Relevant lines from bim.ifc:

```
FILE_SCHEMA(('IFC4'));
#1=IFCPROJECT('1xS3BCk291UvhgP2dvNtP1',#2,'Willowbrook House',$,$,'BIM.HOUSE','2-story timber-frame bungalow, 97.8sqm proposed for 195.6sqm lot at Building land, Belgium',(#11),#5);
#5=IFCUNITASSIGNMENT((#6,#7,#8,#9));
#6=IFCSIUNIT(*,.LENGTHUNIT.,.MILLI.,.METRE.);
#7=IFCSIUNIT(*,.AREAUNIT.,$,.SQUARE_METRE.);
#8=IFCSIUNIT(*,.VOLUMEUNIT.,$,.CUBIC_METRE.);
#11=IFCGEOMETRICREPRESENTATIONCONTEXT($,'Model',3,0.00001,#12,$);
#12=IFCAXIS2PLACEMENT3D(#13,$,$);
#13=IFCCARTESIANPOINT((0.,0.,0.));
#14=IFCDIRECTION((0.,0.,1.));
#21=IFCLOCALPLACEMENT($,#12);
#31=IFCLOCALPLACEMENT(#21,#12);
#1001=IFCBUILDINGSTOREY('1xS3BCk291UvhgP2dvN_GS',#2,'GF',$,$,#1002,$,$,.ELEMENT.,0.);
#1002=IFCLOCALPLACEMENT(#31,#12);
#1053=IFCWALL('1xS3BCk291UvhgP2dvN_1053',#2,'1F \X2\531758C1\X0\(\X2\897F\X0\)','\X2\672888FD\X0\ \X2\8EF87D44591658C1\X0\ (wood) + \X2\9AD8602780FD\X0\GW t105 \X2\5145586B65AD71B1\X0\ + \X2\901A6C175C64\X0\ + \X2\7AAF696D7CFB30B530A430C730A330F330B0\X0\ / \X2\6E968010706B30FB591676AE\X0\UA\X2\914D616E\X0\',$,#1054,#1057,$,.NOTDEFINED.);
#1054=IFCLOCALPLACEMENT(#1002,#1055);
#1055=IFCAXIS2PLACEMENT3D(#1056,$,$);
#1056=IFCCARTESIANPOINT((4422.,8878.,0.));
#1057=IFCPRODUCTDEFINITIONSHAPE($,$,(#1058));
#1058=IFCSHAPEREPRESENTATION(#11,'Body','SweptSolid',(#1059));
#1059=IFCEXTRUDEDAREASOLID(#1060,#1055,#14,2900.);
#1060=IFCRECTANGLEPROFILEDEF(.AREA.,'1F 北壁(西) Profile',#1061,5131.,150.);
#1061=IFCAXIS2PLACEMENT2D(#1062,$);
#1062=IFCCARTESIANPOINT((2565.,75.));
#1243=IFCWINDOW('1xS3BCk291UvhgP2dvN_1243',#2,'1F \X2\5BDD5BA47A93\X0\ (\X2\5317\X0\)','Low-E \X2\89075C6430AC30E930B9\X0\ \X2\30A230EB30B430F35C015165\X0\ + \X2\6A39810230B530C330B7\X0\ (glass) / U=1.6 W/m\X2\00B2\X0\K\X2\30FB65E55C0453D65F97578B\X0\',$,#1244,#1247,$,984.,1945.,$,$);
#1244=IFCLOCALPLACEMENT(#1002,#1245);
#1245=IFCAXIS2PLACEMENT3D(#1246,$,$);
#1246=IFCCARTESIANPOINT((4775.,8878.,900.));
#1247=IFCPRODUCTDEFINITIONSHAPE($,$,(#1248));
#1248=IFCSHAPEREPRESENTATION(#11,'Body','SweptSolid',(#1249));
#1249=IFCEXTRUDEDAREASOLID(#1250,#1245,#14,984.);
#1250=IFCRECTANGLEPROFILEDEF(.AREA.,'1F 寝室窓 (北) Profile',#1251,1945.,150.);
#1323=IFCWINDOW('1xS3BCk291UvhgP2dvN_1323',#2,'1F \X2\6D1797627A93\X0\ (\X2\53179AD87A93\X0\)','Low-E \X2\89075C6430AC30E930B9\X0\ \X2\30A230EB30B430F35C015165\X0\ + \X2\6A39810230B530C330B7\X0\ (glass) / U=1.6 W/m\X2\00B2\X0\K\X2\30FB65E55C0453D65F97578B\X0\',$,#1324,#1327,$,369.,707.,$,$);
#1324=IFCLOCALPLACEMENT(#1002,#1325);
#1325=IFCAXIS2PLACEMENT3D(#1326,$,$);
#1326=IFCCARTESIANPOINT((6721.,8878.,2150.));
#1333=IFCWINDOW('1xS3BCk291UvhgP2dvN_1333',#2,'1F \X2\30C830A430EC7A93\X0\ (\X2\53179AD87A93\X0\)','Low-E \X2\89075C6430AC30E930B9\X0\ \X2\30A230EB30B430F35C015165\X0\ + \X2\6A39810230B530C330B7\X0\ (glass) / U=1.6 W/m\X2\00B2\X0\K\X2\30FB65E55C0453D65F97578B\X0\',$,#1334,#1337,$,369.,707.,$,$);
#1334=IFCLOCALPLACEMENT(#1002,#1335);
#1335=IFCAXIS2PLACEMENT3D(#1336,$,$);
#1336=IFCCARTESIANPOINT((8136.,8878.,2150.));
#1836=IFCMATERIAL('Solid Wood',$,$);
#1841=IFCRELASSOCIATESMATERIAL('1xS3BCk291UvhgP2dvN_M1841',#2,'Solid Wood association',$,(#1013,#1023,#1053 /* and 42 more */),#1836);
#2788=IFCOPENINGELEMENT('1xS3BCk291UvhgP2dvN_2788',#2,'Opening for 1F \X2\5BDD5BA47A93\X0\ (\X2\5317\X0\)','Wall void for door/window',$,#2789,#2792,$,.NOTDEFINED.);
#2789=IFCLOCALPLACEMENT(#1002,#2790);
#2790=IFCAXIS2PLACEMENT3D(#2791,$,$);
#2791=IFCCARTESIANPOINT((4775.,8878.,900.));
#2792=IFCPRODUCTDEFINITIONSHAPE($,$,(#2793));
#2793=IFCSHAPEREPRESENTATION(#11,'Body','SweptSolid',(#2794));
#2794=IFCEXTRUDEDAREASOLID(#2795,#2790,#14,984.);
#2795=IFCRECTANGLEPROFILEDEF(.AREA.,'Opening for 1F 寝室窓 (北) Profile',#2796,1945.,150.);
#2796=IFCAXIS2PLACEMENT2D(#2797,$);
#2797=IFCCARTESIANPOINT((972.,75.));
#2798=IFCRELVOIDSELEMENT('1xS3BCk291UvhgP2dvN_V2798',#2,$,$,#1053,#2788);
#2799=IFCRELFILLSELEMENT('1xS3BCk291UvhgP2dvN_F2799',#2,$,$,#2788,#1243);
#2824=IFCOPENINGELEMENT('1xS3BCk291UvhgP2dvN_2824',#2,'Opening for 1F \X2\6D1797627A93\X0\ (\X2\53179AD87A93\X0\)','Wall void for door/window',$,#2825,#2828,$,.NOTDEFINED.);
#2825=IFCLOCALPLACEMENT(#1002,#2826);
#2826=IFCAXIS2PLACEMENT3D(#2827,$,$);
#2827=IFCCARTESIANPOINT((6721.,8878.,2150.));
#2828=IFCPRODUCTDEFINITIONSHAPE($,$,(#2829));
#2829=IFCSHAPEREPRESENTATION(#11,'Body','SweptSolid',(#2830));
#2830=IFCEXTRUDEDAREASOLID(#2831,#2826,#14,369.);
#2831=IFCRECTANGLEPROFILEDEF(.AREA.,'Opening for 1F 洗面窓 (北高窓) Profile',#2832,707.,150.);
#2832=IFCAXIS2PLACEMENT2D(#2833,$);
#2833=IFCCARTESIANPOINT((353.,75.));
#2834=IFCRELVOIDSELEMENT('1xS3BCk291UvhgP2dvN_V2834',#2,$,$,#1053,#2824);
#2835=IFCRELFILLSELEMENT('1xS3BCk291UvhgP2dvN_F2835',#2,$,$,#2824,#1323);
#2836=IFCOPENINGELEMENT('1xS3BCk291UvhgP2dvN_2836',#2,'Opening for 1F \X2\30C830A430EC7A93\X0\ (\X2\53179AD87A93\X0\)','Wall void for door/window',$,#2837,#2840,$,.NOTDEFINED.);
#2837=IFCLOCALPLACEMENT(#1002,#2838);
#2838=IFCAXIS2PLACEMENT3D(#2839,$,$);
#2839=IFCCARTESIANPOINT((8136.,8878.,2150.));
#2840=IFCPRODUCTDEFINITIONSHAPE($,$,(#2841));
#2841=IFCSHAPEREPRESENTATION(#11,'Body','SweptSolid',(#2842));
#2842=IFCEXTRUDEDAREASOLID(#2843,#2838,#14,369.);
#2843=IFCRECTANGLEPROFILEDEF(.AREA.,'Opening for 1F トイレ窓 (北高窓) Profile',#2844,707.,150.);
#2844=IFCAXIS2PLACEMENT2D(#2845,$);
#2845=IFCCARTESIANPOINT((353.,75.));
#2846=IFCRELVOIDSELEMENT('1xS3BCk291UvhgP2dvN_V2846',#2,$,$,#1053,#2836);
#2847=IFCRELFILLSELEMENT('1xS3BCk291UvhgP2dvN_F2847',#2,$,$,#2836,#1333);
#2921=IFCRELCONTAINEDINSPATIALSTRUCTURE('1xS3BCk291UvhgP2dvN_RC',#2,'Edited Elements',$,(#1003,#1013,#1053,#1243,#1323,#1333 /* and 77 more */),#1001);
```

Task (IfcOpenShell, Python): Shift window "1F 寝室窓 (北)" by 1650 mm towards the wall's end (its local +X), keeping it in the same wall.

```python
import ifcopenshell
import ifcopenshell.api.geometry
import ifcopenshell.util.placement

model = ifcopenshell.open("bim.ifc")

window = model.by_id(1243)
opening = window.FillsVoids[0].RelatingOpeningElement
wall = opening.VoidsElements[0].RelatingBuildingElement

wall_matrix = ifcopenshell.util.placement.get_local_placement(wall.ObjectPlacement)
shift = wall_matrix[:3, 0] * 1650.0
before = ifcopenshell.util.placement.get_local_placement(window.ObjectPlacement)[:3, 3].copy()

# The window is not placed relative to its opening, so move both.
for product in (opening, window):
    matrix = ifcopenshell.util.placement.get_local_placement(product.ObjectPlacement)
    matrix[:3, 3] += shift
    ifcopenshell.api.geometry.edit_object_placement(model, product=product, matrix=matrix, is_si=False)

after = ifcopenshell.util.placement.get_local_placement(window.ObjectPlacement)[:3, 3]
print("window moved by", (after - before).round(3) + 0.0)

model.write("bim_updated.ifc")
```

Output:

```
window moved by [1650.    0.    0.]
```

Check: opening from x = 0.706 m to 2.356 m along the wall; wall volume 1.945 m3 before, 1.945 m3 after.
